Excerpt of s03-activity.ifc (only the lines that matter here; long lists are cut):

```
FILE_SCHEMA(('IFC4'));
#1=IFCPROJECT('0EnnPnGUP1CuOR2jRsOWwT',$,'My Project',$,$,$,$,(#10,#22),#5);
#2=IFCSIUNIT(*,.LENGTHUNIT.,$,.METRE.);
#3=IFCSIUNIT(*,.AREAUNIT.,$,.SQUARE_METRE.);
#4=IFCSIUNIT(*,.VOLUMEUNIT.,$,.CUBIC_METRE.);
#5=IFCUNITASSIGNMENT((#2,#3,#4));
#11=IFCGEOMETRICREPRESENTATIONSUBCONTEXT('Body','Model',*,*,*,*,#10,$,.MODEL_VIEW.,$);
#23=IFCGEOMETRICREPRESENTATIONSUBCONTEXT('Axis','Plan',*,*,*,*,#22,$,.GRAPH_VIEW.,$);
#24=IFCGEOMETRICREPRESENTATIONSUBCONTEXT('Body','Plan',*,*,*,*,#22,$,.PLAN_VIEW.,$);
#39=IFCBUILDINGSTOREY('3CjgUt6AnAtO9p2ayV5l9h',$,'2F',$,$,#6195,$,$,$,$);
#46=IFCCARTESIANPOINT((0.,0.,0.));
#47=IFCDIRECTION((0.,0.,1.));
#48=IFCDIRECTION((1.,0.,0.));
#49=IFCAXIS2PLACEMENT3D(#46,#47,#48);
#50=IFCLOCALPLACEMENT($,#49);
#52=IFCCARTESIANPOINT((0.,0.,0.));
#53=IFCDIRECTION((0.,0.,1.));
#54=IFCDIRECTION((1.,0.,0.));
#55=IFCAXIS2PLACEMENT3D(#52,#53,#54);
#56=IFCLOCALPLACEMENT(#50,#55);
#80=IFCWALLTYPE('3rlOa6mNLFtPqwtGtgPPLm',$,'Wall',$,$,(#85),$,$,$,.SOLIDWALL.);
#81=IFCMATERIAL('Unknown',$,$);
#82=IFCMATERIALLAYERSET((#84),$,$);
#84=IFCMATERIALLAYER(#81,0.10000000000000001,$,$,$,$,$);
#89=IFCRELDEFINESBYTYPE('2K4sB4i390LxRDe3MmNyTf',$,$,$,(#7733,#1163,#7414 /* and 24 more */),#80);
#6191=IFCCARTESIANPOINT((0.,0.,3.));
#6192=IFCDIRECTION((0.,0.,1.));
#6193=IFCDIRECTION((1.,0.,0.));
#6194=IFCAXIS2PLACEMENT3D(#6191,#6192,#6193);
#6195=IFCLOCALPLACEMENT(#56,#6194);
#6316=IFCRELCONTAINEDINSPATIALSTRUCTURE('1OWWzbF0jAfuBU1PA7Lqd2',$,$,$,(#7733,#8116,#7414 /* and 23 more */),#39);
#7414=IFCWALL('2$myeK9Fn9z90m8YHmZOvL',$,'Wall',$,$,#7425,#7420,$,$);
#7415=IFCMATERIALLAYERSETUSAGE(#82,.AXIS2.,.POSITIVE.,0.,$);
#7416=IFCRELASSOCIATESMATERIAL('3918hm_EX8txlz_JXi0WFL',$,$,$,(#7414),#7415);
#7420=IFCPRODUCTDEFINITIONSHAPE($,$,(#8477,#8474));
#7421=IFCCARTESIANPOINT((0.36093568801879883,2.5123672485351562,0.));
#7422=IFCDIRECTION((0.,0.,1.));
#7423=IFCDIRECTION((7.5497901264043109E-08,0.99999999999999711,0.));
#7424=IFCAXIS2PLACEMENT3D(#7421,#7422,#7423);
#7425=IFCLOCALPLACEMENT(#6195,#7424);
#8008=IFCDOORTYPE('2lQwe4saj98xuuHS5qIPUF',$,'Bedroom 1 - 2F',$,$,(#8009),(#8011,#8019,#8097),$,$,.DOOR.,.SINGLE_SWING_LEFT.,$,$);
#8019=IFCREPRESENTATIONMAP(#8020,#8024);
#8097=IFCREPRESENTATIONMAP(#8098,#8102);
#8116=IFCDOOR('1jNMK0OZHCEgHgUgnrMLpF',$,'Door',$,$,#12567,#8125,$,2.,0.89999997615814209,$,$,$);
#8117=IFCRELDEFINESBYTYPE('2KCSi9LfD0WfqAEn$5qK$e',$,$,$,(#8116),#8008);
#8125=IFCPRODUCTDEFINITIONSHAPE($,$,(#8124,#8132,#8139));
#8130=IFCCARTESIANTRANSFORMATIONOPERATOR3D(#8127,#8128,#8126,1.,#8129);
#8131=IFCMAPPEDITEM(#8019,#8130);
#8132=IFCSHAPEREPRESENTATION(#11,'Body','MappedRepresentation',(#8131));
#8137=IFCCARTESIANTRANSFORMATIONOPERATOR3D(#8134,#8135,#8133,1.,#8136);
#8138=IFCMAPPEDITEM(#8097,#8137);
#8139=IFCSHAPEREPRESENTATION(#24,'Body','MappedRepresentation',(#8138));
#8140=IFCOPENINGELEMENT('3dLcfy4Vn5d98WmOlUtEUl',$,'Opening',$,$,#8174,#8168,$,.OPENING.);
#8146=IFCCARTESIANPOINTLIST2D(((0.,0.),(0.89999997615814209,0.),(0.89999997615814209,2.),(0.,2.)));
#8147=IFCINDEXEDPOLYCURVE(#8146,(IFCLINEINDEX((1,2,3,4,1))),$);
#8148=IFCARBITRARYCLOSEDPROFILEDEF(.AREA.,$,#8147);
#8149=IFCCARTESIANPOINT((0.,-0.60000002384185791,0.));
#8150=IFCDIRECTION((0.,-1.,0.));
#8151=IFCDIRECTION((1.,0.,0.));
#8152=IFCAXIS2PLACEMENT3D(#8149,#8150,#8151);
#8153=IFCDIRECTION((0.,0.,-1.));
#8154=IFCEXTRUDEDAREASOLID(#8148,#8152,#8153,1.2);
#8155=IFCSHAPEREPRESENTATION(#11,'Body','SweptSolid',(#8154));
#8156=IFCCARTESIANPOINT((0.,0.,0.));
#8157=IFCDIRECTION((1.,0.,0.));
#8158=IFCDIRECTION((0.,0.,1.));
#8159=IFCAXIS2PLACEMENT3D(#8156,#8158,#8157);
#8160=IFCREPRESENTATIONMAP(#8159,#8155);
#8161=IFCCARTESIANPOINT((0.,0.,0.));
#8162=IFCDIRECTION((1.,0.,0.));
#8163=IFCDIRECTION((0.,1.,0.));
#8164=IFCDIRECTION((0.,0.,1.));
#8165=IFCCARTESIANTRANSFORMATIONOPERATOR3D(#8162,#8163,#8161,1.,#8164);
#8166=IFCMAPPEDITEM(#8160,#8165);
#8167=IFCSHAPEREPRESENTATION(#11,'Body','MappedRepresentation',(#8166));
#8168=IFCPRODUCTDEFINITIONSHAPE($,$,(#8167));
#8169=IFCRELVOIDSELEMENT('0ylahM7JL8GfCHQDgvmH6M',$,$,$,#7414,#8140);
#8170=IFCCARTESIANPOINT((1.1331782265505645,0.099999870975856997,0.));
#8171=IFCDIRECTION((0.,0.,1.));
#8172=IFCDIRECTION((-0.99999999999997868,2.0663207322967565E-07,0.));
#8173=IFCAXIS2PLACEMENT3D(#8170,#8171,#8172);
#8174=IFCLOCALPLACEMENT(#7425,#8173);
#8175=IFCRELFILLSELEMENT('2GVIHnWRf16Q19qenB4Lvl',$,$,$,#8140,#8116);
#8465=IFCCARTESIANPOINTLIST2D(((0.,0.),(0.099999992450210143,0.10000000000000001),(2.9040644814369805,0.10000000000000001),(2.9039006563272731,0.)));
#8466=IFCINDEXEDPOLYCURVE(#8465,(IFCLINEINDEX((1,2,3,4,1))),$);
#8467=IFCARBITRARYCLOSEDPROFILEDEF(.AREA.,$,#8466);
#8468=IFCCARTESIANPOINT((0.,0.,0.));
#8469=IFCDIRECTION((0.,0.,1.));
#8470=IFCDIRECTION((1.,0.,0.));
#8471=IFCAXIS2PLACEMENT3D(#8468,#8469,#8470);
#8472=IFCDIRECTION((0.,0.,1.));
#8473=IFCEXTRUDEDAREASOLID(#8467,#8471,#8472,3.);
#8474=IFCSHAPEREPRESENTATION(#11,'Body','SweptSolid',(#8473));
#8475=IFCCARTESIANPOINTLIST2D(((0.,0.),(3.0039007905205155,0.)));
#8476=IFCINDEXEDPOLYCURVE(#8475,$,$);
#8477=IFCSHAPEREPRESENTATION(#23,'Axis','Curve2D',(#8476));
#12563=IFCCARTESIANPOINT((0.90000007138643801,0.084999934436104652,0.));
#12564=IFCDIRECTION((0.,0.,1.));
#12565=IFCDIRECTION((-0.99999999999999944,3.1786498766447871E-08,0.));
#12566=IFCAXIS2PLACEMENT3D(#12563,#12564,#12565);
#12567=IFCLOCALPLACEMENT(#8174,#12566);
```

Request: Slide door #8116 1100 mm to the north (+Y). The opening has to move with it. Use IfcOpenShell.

```python
import ifcopenshell
import ifcopenshell.api.geometry
import ifcopenshell.util.placement

model = ifcopenshell.open("s03-activity.ifc")

door = model.by_id(8116)
opening = door.FillsVoids[0].RelatingOpeningElement
wall = opening.VoidsElements[0].RelatingBuildingElement

wall_matrix = ifcopenshell.util.placement.get_local_placement(wall.ObjectPlacement)
shift = wall_matrix[:3, 0] * 1.1
before = ifcopenshell.util.placement.get_local_placement(door.ObjectPlacement)[:3, 3].copy()

# The door is placed relative to its opening, so it follows when the opening moves.
matrix = ifcopenshell.util.placement.get_local_placement(opening.ObjectPlacement)
matrix[:3, 3] += shift
ifcopenshell.api.geometry.edit_object_placement(
    model, product=opening, matrix=matrix, is_si=False, should_transform_children=True
)

after = ifcopenshell.util.placement.get_local_placement(door.ObjectPlacement)[:3, 3]
print("door moved by", (after - before).round(3) + 0.0)

model.write("s03-activity_rev.ifc")
```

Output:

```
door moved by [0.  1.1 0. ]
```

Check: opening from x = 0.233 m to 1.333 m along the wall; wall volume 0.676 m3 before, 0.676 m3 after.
